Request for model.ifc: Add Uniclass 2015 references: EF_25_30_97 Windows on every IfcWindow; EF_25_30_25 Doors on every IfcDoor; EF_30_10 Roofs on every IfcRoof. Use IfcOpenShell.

First a look at what the model holds.

```python
import ifcopenshell

model = ifcopenshell.open("model.ifc")
print(model.schema)
print("classifications:", [c.Name for c in model.by_type("IfcClassification")])
for ifc_class in ("IfcDoor", "IfcRoof", "IfcStair", "IfcWall", "IfcWindow"):
    print(ifc_class, len(model.by_type(ifc_class)))
```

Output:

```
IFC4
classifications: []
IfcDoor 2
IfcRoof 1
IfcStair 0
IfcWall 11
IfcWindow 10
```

```python
import ifcopenshell
import ifcopenshell.api.classification

model = ifcopenshell.open("model.ifc")

system = ifcopenshell.api.classification.add_classification(model, classification="Uniclass 2015")

codes = {
    "IfcWindow": ("EF_25_30_97", "Windows"),
    "IfcDoor": ("EF_25_30_25", "Doors"),
    "IfcRoof": ("EF_30_10", "Roofs"),
}
for ifc_class, (code, name) in codes.items():
    products = model.by_type(ifc_class)
    ifcopenshell.api.classification.add_reference(
        model, products=products, classification=system, identification=code, name=name
    )
    print(code, len(products))

model.write("model_edited.ifc")
```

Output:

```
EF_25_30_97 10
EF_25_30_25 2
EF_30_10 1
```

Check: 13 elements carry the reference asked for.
